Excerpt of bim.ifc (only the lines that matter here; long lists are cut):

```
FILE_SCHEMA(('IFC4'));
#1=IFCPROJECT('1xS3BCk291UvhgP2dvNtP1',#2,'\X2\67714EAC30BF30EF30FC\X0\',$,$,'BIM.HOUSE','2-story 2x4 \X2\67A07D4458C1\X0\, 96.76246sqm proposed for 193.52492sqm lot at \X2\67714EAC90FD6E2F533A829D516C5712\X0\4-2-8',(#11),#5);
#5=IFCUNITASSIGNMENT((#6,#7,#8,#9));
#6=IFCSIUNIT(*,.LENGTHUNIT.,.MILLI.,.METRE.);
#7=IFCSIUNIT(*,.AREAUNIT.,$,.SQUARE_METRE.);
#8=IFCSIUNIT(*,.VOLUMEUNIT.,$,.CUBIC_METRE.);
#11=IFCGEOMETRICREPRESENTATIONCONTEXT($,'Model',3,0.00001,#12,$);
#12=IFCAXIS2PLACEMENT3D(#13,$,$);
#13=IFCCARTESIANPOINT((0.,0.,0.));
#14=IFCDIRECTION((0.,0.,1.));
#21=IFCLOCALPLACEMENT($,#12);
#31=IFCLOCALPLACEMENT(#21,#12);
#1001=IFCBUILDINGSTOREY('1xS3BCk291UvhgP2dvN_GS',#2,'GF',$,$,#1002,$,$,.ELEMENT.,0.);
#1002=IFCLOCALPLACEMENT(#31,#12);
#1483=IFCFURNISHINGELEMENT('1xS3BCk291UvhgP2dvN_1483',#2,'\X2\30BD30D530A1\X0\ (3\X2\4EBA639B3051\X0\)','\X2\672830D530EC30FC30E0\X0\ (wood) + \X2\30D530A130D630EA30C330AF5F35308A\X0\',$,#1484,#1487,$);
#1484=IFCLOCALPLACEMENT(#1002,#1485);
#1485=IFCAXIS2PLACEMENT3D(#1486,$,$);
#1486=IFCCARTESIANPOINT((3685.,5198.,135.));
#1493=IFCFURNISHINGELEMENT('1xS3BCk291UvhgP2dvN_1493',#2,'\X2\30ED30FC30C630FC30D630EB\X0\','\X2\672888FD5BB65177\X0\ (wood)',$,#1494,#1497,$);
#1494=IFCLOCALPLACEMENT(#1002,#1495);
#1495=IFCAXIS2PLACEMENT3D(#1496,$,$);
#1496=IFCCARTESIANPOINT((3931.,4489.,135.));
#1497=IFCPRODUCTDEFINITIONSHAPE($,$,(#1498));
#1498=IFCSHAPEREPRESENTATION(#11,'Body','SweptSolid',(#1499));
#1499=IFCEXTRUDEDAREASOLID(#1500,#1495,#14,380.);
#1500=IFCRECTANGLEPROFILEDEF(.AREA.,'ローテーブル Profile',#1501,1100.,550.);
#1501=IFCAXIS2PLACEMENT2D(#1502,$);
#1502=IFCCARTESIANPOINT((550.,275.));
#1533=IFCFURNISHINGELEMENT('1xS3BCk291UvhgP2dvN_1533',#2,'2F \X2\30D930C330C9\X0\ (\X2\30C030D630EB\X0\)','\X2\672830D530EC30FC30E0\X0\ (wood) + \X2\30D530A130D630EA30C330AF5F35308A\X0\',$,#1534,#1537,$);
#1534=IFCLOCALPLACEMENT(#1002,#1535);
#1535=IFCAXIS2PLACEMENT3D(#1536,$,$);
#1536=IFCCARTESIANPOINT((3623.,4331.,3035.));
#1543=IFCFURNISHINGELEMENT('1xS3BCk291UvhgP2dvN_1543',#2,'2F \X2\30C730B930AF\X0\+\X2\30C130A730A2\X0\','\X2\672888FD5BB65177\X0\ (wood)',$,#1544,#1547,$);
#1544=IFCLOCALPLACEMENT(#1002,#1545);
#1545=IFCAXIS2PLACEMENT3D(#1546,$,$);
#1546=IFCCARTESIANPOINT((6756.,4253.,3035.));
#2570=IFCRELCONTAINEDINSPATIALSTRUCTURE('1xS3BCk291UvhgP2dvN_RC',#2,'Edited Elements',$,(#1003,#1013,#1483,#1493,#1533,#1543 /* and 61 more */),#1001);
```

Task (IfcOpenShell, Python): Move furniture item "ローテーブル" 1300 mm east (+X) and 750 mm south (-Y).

```python
import ifcopenshell
import ifcopenshell.api.geometry
import ifcopenshell.util.placement
import ifcopenshell.util.unit

model = ifcopenshell.open("bim.ifc")
unit_scale = ifcopenshell.util.unit.calculate_unit_scale(model)

item = model.by_guid("1xS3BCk291UvhgP2dvN_1493")
matrix = ifcopenshell.util.placement.get_local_placement(item.ObjectPlacement)
matrix[0, 3] += 1.3 / unit_scale
matrix[1, 3] -= 0.75 / unit_scale
ifcopenshell.api.geometry.edit_object_placement(model, product=item, matrix=matrix, is_si=False)

print(ifcopenshell.util.placement.get_local_placement(item.ObjectPlacement).round(3) + 0.0)

model.write("bim_v2.ifc")
```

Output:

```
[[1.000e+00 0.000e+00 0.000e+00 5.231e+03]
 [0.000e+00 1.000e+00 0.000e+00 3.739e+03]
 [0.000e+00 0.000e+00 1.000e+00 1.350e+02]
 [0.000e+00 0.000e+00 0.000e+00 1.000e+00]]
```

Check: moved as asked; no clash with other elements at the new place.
